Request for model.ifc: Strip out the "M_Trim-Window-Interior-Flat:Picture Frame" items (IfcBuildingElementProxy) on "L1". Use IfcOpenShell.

First a look at what the model holds.

```python
import ifcopenshell
import ifcopenshell.util.element

model = ifcopenshell.open("model.ifc")
print(model.schema)
storey = next(s for s in model.by_type("IfcBuildingStorey") if s.Name == "L1")
proxies = [e for e in ifcopenshell.util.element.get_decomposition(storey) if e.is_a("IfcBuildingElementProxy")]
seen = {}
for e in proxies:
    element_type = ifcopenshell.util.element.get_type(e)
    name = element_type.Name if element_type not in (None, e) else None
    seen[name] = seen.get(name, 0) + 1
for name, count in sorted(seen.items(), key=str):
    print(count, "x", name)
```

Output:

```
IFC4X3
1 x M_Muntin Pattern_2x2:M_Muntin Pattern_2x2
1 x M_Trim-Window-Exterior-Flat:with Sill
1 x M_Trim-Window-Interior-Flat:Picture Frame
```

```python
import ifcopenshell
import ifcopenshell.api.root
import ifcopenshell.util.element

model = ifcopenshell.open("model.ifc")

storey = next(s for s in model.by_type("IfcBuildingStorey") if s.Name == "L1")
proxies = [e for e in ifcopenshell.util.element.get_decomposition(storey) if e.is_a("IfcBuildingElementProxy")]
targets = [e for e in proxies if (t := ifcopenshell.util.element.get_type(e)) not in (None, e) and t.Name == "M_Trim-Window-Interior-Flat:Picture Frame"]

for e in targets:
    ifcopenshell.api.root.remove_product(model, product=e)
print(len(targets), "removed")

model.write("model_v2.ifc")
```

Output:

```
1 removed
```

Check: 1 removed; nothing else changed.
